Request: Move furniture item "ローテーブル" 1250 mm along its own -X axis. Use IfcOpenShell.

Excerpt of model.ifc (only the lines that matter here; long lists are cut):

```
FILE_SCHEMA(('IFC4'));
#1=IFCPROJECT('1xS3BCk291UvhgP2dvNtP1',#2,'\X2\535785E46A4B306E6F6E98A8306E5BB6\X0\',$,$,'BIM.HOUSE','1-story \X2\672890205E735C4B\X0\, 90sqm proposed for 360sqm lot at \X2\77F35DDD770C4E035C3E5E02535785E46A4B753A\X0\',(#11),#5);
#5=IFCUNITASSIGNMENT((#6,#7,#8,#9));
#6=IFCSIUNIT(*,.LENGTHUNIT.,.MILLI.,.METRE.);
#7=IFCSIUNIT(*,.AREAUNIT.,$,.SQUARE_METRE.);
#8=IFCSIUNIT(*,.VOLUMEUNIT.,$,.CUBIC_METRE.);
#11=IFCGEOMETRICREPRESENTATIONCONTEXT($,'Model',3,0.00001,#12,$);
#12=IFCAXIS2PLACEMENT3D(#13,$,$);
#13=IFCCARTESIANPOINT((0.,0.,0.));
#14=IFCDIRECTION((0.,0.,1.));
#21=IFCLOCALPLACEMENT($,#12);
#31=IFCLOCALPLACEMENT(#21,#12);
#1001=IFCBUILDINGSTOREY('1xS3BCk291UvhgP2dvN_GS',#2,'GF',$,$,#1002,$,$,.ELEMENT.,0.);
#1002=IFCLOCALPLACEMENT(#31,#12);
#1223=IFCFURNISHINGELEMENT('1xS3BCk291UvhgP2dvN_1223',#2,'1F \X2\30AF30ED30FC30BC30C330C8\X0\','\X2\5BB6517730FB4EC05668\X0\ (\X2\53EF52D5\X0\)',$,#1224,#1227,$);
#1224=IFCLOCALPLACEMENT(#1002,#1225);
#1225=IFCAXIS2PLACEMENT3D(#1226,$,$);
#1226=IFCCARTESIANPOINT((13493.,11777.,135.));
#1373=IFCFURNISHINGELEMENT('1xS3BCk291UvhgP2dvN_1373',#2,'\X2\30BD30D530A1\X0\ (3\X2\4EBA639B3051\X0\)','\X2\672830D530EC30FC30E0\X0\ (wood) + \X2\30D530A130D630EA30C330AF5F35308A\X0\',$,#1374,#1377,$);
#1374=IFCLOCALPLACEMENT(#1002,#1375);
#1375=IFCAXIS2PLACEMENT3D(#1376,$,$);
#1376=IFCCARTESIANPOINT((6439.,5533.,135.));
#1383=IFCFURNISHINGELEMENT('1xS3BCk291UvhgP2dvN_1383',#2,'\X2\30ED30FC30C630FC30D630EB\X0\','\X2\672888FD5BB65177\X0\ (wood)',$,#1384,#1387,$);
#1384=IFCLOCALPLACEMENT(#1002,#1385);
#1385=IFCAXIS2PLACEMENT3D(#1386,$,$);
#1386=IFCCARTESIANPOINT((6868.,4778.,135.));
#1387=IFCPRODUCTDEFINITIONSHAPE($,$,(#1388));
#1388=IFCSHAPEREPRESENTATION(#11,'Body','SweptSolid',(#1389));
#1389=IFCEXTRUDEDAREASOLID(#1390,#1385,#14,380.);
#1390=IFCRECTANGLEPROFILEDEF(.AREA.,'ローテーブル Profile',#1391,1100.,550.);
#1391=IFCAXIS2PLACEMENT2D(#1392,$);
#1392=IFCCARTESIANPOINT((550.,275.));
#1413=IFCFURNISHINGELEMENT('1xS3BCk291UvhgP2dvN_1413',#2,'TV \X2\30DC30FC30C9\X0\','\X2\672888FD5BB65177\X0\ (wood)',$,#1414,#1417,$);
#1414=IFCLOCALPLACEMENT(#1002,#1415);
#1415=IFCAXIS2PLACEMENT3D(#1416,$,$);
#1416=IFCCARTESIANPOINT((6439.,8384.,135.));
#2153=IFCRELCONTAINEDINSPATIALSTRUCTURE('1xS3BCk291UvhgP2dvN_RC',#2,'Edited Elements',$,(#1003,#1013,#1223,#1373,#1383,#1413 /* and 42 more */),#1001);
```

```python
import ifcopenshell
import ifcopenshell.api.geometry
import ifcopenshell.util.placement

model = ifcopenshell.open("model.ifc")

item = model.by_guid("1xS3BCk291UvhgP2dvN_1383")
matrix = ifcopenshell.util.placement.get_local_placement(item.ObjectPlacement)
matrix[:3, 3] -= matrix[:3, 0] * 1250.0
ifcopenshell.api.geometry.edit_object_placement(model, product=item, matrix=matrix, is_si=False)

print(ifcopenshell.util.placement.get_local_placement(item.ObjectPlacement).round(3) + 0.0)

model.write("model_rev.ifc")
```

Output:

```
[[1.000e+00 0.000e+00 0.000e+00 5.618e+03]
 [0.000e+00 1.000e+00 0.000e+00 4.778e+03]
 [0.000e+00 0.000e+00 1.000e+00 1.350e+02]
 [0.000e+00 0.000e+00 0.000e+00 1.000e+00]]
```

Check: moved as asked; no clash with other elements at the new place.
